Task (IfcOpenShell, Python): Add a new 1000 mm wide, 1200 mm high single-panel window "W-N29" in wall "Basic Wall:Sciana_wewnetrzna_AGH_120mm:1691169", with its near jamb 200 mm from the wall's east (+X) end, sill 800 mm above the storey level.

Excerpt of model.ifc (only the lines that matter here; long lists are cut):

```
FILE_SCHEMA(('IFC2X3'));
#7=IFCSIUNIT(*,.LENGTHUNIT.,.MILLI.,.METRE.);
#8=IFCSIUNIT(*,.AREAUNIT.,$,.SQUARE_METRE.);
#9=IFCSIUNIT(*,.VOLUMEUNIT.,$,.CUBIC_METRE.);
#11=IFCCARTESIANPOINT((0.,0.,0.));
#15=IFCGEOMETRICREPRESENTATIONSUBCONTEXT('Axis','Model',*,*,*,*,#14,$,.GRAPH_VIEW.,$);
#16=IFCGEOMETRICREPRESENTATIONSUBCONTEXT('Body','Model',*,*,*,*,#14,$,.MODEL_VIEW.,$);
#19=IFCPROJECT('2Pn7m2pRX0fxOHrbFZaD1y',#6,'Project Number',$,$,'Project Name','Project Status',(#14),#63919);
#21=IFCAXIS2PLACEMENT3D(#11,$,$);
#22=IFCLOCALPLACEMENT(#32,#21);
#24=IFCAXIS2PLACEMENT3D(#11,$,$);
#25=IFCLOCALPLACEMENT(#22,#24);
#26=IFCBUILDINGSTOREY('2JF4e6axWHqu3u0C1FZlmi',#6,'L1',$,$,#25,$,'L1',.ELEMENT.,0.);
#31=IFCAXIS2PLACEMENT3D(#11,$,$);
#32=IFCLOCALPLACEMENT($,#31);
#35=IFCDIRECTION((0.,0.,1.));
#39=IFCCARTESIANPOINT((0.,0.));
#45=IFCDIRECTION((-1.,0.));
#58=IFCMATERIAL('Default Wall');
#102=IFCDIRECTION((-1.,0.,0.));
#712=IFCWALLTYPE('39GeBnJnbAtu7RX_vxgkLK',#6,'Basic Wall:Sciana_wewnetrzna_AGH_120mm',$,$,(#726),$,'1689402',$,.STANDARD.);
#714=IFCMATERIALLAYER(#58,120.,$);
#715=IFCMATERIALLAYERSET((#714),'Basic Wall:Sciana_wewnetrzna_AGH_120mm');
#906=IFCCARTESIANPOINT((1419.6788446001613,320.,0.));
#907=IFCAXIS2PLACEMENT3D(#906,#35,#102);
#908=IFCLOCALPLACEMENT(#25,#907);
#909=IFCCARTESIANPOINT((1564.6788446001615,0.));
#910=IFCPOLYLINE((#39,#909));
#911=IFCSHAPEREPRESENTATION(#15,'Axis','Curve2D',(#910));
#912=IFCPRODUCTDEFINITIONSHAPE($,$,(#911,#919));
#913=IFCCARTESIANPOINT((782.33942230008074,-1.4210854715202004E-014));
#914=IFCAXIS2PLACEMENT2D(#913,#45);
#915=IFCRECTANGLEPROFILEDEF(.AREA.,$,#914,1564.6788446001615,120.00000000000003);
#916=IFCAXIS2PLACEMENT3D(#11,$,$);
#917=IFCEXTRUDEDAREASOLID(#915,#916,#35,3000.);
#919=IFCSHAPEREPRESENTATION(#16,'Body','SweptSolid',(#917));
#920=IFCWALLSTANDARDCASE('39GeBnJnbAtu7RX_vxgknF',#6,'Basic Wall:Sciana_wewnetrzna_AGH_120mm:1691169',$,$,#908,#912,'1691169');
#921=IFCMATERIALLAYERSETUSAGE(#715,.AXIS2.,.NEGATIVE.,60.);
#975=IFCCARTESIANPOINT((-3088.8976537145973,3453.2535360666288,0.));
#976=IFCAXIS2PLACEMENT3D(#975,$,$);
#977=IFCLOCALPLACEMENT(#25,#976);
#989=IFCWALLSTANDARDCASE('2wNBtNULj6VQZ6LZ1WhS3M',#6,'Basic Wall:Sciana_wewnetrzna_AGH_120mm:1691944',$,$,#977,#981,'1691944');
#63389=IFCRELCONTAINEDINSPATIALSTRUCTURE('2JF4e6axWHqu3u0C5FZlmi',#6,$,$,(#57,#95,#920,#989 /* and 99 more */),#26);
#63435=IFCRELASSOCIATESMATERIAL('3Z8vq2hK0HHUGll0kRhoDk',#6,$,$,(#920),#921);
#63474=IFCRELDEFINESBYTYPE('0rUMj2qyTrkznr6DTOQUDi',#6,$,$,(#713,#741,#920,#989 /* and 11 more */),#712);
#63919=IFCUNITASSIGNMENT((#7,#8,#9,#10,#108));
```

```python
import numpy as np
import ifcopenshell
import ifcopenshell.api.feature
import ifcopenshell.api.geometry
import ifcopenshell.api.root
import ifcopenshell.api.spatial
import ifcopenshell.api.type
import ifcopenshell.geom
import ifcopenshell.util.element
import ifcopenshell.util.placement
import ifcopenshell.util.representation
import ifcopenshell.util.shape
import ifcopenshell.util.unit

model = ifcopenshell.open("model.ifc")
unit_scale = ifcopenshell.util.unit.calculate_unit_scale(model)
settings = ifcopenshell.geom.settings()


def volume(element):
    """Net volume in cubic metres, openings subtracted."""
    shape = ifcopenshell.geom.create_shape(settings, element)
    return ifcopenshell.util.shape.get_volume(shape.geometry)


wall = model.by_guid("39GeBnJnbAtu7RX_vxgknF")
storey = ifcopenshell.util.element.get_container(wall, ifc_class="IfcBuildingStorey")
context = ifcopenshell.util.representation.get_context(model, "Model", "Body", "MODEL_VIEW")
before = volume(wall)

width, height, from_end, sill = 1, 1.2, 0.2, 0.8  # metres

# The wall runs along its own X axis, and the end named is its -X end.
wall_shape = ifcopenshell.geom.create_shape(settings, wall)
x, y, z = ifcopenshell.util.shape.get_vertices(wall_shape.geometry).T
start = x.min() + from_end
face, thickness = float(y.min()), float(y.max() - y.min())
wall_matrix = ifcopenshell.util.placement.get_local_placement(wall.ObjectPlacement)
level = ifcopenshell.util.placement.get_local_placement(storey.ObjectPlacement)[2, 3]


def in_wall(x, y):
    """Placement at x, y metres in the wall's axes, at sill height."""
    matrix = wall_matrix.copy()
    matrix[:, 3] = wall_matrix @ np.array([x / unit_scale, y / unit_scale, 0.0, 1.0])
    matrix[2, 3] = level + sill / unit_scale
    return matrix


# Opening: a box that overshoots both wall faces by 50 mm.
opening = ifcopenshell.api.root.create_entity(model, ifc_class="IfcOpeningElement")
box = ifcopenshell.api.geometry.add_wall_representation(
    model, context=context, length=width, height=height, thickness=thickness + 0.1
)
ifcopenshell.api.geometry.assign_representation(model, product=opening, representation=box)
ifcopenshell.api.geometry.edit_object_placement(model, product=opening, matrix=in_wall(start, face - 0.05), is_si=False)
ifcopenshell.api.feature.add_feature(model, feature=opening, element=wall)

window = ifcopenshell.api.root.create_entity(model, ifc_class="IfcWindow", name="W-N29")
window.OverallWidth, window.OverallHeight = width / unit_scale, height / unit_scale
body = ifcopenshell.api.geometry.add_window_representation(
    model,
    context=context,
    overall_width=window.OverallWidth,
    overall_height=window.OverallHeight,
    partition_type="SINGLE_PANEL",
)
ifcopenshell.api.geometry.assign_representation(model, product=window, representation=body)
ifcopenshell.api.spatial.assign_container(model, products=[window], relating_structure=storey)
fills = ifcopenshell.api.feature.add_filling(model, opening=opening, element=window)
fills.OwnerHistory = window.OwnerHistory  # required in IFC2X3

# IFC2X3 keeps the operation on the window style.
style = ifcopenshell.api.root.create_entity(model, ifc_class="IfcWindowStyle", name="W-N29")
style.OperationType, style.ConstructionType = "SINGLE_PANEL", "NOTDEFINED"
style.ParameterTakesPrecedence = style.Sizeable = False
ifcopenshell.api.type.assign_type(model, related_objects=[window], relating_type=style)

# Centre the window in the wall's thickness.
ifcopenshell.api.geometry.edit_object_placement(model, product=window, matrix=in_wall(start, face), is_si=False)
window_shape = ifcopenshell.geom.create_shape(settings, window)
depth = ifcopenshell.util.shape.get_vertices(window_shape.geometry)[:, 1]
offset = face + thickness / 2 - (depth.min() + depth.max()) / 2
ifcopenshell.api.geometry.edit_object_placement(model, product=window, matrix=in_wall(start, offset), is_si=False)

after = volume(wall)

print(f"wall volume {before:.3f} -> {after:.3f} m3")

model.write("model_v2.ifc")
```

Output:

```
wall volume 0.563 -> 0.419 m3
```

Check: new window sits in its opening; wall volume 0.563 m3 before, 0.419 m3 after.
